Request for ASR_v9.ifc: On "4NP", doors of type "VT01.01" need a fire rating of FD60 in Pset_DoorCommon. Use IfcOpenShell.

First a look at what the model holds.

```python
import ifcopenshell
import ifcopenshell.util.element

model = ifcopenshell.open("ASR_v9.ifc")
print(model.schema)
storey = next(s for s in model.by_type("IfcBuildingStorey") if s.Name == "4NP")
doors = [e for e in ifcopenshell.util.element.get_decomposition(storey) if e.is_a("IfcDoor")]
seen = {}
for e in doors:
    element_type = ifcopenshell.util.element.get_type(e)
    key = (element_type.Name if element_type != e and element_type else None, ifcopenshell.util.element.get_pset(e, "Pset_DoorCommon", "FireRating"))
    seen[key] = seen.get(key, 0) + 1
for (name, value), count in sorted(seen.items(), key=str):
    print(count, "x", name, "|", value)
```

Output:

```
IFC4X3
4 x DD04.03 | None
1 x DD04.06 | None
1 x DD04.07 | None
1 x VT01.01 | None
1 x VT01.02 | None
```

```python
import ifcopenshell
import ifcopenshell.api.pset
import ifcopenshell.util.element

model = ifcopenshell.open("ASR_v9.ifc")

storey = next(s for s in model.by_type("IfcBuildingStorey") if s.Name == "4NP")
doors = [e for e in ifcopenshell.util.element.get_decomposition(storey) if e.is_a("IfcDoor")]

count = 0
for e in doors:
    element_type = ifcopenshell.util.element.get_type(e)
    if element_type in (None, e) or element_type.Name != "VT01.01":
        continue
    # add_pset returns the element's existing set when there is one.
    pset = ifcopenshell.api.pset.add_pset(model, product=e, name="Pset_DoorCommon")
    ifcopenshell.api.pset.edit_pset(model, pset=pset, properties={"FireRating": "FD60"})
    count += 1

print(count, "doors updated")

model.write("ASR_v9-out.ifc")
```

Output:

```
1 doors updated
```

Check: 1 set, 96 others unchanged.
